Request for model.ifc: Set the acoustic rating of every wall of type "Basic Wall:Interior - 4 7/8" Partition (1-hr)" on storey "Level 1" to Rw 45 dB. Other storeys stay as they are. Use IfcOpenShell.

First a look at what the model holds.

```python
import ifcopenshell
import ifcopenshell.util.element

model = ifcopenshell.open("model.ifc")
print(model.schema)
storey = next(s for s in model.by_type("IfcBuildingStorey") if s.Name == "Level 1")
walls = [e for e in ifcopenshell.util.element.get_decomposition(storey) if e.is_a("IfcWall")]
seen = {}
for e in walls:
    element_type = ifcopenshell.util.element.get_type(e)
    key = (element_type.Name if element_type != e and element_type else None, ifcopenshell.util.element.get_pset(e, "Pset_WallCommon", "AcousticRating"))
    seen[key] = seen.get(key, 0) + 1
for (name, value), count in sorted(seen.items(), key=str):
    print(count, "x", name, "|", value)
```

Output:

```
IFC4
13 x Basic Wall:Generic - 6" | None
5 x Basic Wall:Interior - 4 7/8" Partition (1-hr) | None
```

```python
import ifcopenshell
import ifcopenshell.api.pset
import ifcopenshell.util.element

model = ifcopenshell.open("model.ifc")

storey = next(s for s in model.by_type("IfcBuildingStorey") if s.Name == "Level 1")
walls = [e for e in ifcopenshell.util.element.get_decomposition(storey) if e.is_a("IfcWall")]

count = 0
for e in walls:
    element_type = ifcopenshell.util.element.get_type(e)
    if element_type in (None, e) or element_type.Name != 'Basic Wall:Interior - 4 7/8" Partition (1-hr)':
        continue
    # add_pset returns the element's existing set when there is one.
    pset = ifcopenshell.api.pset.add_pset(model, product=e, name="Pset_WallCommon")
    ifcopenshell.api.pset.edit_pset(model, pset=pset, properties={"AcousticRating": "Rw 45 dB"})
    count += 1

print(count, "walls updated")

model.write("model_edited.ifc")
```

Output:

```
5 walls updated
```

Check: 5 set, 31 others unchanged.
